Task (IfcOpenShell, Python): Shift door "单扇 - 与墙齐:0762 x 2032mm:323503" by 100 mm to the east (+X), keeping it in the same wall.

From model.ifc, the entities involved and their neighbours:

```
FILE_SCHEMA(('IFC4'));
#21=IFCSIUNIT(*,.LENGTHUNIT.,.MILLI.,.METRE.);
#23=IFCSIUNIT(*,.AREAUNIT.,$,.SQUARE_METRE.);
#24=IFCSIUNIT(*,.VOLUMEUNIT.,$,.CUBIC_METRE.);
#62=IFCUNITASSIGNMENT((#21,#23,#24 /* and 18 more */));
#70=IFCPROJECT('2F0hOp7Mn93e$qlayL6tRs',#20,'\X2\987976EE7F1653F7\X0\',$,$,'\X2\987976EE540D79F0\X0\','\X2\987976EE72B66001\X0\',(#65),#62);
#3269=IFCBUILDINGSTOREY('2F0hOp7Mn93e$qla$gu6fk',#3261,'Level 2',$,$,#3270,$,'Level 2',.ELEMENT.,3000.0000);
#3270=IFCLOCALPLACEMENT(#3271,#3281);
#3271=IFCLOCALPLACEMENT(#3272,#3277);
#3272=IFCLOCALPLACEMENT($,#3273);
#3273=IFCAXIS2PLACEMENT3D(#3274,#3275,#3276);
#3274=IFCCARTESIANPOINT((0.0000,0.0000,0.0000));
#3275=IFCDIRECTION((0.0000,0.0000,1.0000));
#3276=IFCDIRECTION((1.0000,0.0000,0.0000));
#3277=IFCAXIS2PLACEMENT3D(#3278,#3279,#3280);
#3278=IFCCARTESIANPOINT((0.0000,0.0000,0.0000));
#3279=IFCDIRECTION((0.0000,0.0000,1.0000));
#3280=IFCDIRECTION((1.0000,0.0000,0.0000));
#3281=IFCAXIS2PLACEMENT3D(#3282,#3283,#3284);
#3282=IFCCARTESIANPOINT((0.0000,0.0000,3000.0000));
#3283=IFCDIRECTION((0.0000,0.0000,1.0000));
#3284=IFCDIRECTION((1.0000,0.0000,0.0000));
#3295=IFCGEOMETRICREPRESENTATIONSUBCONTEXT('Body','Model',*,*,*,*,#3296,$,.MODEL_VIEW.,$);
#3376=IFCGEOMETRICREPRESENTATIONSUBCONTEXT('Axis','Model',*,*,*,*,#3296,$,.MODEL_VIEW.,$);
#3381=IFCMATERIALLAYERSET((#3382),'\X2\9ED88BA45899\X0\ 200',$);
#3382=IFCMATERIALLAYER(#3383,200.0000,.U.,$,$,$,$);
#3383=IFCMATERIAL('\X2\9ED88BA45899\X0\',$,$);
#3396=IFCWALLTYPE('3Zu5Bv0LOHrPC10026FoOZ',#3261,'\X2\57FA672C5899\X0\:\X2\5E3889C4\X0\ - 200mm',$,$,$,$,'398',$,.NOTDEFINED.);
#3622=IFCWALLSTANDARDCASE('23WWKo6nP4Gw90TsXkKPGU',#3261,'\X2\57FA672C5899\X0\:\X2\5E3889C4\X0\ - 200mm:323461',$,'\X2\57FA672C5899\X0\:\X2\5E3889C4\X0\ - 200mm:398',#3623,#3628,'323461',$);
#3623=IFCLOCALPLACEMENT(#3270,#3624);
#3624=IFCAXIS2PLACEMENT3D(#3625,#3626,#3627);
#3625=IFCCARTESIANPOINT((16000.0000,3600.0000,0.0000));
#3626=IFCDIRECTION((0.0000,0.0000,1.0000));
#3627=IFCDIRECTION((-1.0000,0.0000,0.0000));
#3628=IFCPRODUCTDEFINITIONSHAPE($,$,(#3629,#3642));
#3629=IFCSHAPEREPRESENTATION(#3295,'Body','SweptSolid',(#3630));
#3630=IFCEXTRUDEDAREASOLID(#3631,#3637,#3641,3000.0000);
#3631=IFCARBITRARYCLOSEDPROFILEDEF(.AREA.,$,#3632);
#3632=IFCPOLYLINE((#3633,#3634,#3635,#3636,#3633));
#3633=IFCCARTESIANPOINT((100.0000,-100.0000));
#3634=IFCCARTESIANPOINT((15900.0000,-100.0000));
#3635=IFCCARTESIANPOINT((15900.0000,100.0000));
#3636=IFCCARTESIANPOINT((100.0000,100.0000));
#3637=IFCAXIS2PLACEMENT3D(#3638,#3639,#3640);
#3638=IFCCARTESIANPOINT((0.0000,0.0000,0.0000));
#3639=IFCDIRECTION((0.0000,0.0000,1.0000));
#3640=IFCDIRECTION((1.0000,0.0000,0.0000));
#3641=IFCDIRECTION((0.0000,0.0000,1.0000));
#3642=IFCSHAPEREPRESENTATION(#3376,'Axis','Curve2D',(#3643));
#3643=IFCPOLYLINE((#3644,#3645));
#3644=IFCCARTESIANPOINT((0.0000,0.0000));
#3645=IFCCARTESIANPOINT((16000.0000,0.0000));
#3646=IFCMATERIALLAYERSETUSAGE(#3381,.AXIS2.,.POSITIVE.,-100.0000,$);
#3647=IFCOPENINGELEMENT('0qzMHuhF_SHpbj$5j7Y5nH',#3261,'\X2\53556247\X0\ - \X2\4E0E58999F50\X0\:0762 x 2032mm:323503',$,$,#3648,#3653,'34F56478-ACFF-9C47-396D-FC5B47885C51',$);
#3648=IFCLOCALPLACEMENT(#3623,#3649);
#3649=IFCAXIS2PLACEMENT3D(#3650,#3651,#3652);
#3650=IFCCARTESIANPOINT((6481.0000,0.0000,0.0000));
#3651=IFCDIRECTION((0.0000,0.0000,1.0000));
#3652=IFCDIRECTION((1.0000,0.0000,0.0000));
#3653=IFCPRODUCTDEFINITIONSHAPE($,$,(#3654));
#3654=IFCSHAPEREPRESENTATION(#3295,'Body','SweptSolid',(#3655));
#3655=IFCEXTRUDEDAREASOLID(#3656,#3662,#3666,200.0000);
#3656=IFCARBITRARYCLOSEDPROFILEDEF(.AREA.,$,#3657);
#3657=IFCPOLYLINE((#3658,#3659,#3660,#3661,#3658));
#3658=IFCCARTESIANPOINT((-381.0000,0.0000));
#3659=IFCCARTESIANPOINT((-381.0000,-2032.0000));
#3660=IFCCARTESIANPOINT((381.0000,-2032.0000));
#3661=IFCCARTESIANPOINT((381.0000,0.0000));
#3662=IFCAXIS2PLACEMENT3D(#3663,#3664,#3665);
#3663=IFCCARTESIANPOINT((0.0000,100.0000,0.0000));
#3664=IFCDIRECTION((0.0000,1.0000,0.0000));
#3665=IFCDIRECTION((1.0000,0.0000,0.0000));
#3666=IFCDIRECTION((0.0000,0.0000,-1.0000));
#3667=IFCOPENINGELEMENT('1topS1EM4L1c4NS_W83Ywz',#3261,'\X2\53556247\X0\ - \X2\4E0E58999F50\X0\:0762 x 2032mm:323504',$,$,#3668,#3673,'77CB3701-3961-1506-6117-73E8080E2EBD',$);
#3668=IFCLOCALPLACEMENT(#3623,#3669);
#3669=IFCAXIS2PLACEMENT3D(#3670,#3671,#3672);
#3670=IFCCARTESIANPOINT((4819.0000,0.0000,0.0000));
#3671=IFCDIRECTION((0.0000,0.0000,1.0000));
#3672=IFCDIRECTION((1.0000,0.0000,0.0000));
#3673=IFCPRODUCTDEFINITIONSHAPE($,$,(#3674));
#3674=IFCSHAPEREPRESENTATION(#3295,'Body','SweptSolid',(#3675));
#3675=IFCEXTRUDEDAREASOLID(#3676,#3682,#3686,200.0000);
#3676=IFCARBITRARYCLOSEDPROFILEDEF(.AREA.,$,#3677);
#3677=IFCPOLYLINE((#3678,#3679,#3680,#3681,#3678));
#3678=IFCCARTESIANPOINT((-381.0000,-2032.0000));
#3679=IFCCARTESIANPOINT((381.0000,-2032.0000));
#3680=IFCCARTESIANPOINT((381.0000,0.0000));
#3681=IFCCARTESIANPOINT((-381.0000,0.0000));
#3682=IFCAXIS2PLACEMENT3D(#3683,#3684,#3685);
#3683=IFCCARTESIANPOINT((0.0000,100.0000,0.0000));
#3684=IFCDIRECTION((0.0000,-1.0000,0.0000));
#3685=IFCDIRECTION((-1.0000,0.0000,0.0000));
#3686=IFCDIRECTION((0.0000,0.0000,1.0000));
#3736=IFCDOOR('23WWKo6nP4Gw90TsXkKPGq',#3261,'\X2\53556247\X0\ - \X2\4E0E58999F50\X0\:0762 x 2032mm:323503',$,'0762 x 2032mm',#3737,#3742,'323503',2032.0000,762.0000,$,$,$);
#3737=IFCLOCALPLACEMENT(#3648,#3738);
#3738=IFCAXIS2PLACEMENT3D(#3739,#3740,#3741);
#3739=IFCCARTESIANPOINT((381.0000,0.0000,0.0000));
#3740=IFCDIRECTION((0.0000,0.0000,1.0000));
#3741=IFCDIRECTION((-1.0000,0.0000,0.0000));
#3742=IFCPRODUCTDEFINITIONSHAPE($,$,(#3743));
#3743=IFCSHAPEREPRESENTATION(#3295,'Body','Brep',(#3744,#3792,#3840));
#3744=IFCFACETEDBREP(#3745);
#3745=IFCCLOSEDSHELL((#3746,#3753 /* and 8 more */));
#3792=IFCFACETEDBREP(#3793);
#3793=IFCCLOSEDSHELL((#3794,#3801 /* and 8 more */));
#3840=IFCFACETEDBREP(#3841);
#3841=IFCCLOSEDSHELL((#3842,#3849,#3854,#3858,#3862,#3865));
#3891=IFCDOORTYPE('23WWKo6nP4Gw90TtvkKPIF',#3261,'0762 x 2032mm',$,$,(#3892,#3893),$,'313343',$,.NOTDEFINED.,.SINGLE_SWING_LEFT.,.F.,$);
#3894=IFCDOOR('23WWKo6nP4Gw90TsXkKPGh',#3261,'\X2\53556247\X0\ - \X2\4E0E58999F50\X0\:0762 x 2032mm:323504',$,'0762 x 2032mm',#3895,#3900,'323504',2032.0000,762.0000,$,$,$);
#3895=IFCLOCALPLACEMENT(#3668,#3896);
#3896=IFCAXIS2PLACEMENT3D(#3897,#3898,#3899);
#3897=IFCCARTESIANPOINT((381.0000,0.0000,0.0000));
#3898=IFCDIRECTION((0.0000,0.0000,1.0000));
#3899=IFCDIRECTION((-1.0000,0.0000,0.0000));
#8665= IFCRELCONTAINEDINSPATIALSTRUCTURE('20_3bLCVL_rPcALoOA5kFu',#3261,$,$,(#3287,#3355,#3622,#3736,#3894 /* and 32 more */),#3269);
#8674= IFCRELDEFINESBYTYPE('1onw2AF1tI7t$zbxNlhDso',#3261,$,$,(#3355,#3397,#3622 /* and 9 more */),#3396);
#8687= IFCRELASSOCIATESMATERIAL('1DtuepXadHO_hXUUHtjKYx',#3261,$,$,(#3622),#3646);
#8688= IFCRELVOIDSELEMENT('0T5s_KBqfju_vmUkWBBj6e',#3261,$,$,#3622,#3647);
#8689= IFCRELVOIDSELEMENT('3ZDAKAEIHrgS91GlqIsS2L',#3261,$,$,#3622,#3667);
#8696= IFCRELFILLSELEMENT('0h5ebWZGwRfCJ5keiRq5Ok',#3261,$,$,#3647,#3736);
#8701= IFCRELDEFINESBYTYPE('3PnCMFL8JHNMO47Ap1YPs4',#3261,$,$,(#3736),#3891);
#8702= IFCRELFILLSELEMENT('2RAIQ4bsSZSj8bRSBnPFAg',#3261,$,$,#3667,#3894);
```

```python
import ifcopenshell
import ifcopenshell.api.geometry
import ifcopenshell.util.placement
import ifcopenshell.util.unit

model = ifcopenshell.open("model.ifc")
unit_scale = ifcopenshell.util.unit.calculate_unit_scale(model)

door = model.by_guid("23WWKo6nP4Gw90TsXkKPGq")
opening = door.FillsVoids[0].RelatingOpeningElement
wall = opening.VoidsElements[0].RelatingBuildingElement

wall_matrix = ifcopenshell.util.placement.get_local_placement(wall.ObjectPlacement)
shift = wall_matrix[:3, 0] * -0.1 / unit_scale
before = ifcopenshell.util.placement.get_local_placement(door.ObjectPlacement)[:3, 3].copy()

# The door is placed relative to its opening, so it follows when the opening moves.
matrix = ifcopenshell.util.placement.get_local_placement(opening.ObjectPlacement)
matrix[:3, 3] += shift
ifcopenshell.api.geometry.edit_object_placement(
    model, product=opening, matrix=matrix, is_si=False, should_transform_children=True
)

after = ifcopenshell.util.placement.get_local_placement(door.ObjectPlacement)[:3, 3]
print("door moved by", (after - before).round(3) + 0.0)

model.write("model_rev.ifc")
```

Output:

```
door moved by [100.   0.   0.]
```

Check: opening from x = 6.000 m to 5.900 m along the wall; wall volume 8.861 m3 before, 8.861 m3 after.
